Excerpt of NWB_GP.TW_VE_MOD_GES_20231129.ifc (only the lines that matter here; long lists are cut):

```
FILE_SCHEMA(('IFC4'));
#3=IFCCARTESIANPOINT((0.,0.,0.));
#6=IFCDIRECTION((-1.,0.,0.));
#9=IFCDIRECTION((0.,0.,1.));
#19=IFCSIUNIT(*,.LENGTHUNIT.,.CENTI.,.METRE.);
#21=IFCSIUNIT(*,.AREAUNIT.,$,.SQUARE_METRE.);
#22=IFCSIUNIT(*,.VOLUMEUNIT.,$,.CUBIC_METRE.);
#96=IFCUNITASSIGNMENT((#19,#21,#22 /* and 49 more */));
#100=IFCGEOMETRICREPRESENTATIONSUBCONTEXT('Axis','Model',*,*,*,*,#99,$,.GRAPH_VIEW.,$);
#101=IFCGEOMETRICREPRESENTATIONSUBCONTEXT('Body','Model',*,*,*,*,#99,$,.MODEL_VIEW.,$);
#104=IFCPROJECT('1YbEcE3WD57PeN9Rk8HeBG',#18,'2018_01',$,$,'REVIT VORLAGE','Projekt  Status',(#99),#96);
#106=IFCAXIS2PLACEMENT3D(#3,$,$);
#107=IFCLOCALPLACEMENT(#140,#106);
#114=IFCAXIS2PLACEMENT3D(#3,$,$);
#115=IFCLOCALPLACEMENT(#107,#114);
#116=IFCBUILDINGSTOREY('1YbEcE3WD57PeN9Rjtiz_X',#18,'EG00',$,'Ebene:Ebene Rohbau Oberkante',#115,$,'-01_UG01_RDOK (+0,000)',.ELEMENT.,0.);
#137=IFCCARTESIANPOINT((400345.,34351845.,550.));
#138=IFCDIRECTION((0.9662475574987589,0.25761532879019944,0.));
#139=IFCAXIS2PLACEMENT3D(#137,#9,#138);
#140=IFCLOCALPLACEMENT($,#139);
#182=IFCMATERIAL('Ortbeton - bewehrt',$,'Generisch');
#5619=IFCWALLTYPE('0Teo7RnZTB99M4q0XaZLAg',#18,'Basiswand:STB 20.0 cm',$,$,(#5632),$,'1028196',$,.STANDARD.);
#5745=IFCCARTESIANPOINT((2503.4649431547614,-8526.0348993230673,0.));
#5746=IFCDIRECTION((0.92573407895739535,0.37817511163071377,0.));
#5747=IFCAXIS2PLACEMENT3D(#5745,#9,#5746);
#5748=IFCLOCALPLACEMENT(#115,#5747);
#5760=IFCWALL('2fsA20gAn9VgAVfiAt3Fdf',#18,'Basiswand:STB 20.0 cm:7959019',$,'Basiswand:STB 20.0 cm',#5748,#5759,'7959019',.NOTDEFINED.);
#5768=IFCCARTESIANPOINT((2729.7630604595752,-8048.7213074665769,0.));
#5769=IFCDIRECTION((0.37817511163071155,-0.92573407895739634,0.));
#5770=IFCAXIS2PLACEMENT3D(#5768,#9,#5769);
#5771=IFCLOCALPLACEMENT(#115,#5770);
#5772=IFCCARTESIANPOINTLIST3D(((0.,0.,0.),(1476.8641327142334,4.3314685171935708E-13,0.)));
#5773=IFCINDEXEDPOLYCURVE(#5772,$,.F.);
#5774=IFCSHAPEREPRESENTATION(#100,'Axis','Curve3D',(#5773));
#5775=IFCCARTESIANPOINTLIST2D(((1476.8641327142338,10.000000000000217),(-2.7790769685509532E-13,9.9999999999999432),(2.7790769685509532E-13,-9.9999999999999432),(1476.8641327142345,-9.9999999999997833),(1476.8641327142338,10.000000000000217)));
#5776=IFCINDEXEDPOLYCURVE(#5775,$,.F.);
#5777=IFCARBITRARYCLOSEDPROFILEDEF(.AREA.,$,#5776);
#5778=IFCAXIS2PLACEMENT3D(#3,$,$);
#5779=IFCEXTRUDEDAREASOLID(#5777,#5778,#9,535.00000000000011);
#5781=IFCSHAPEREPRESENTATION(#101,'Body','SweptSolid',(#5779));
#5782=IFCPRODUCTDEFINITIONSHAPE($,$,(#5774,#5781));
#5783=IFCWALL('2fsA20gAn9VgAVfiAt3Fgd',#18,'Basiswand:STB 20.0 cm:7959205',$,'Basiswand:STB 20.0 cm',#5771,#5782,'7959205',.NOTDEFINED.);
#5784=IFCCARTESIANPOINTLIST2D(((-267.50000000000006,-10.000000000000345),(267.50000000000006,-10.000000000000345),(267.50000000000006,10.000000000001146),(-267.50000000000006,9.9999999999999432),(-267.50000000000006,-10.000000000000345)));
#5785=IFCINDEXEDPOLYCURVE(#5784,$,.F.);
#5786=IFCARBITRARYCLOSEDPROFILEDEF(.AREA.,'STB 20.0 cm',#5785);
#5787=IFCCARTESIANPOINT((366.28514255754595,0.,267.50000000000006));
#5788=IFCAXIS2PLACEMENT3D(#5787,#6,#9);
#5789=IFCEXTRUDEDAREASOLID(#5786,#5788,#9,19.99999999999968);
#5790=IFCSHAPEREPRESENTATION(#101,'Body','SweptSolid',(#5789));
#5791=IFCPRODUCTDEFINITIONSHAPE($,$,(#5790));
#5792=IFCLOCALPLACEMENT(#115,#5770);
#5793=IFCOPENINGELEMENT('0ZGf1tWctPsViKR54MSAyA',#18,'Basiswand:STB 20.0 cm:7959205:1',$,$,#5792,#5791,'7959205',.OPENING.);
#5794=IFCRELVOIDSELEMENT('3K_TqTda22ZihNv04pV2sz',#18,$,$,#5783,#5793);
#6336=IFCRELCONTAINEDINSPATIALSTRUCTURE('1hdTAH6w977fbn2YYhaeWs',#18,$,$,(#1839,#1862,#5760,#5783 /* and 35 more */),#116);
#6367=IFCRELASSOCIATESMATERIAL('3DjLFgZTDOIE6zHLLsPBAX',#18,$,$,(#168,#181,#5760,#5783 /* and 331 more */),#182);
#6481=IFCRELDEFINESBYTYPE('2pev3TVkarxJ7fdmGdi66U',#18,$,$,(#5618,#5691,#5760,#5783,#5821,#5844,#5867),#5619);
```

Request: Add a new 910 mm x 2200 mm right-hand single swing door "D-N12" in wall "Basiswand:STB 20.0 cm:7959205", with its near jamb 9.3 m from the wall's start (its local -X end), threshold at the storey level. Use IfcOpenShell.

```python
import numpy as np
import ifcopenshell
import ifcopenshell.api.feature
import ifcopenshell.api.geometry
import ifcopenshell.api.root
import ifcopenshell.api.spatial
import ifcopenshell.geom
import ifcopenshell.util.element
import ifcopenshell.util.placement
import ifcopenshell.util.representation
import ifcopenshell.util.shape
import ifcopenshell.util.unit

model = ifcopenshell.open("NWB_GP.TW_VE_MOD_GES_20231129.ifc")
unit_scale = ifcopenshell.util.unit.calculate_unit_scale(model)
settings = ifcopenshell.geom.settings()


def volume(element):
    """Net volume in cubic metres, openings subtracted."""
    shape = ifcopenshell.geom.create_shape(settings, element)
    return ifcopenshell.util.shape.get_volume(shape.geometry)


wall = model.by_guid("2fsA20gAn9VgAVfiAt3Fgd")
storey = ifcopenshell.util.element.get_container(wall, ifc_class="IfcBuildingStorey")
context = ifcopenshell.util.representation.get_context(model, "Model", "Body", "MODEL_VIEW")
before = volume(wall)

width, height, from_end, sill = 0.91, 2.2, 9.3, 0.0  # metres

# The wall runs along its own X axis, and the end named is its -X end.
wall_shape = ifcopenshell.geom.create_shape(settings, wall)
x, y, z = ifcopenshell.util.shape.get_vertices(wall_shape.geometry).T
start = x.min() + from_end
face, thickness = float(y.min()), float(y.max() - y.min())
wall_matrix = ifcopenshell.util.placement.get_local_placement(wall.ObjectPlacement)
level = ifcopenshell.util.placement.get_local_placement(storey.ObjectPlacement)[2, 3]


def in_wall(x, y):
    """Placement at x, y metres in the wall's axes, at sill height."""
    matrix = wall_matrix.copy()
    matrix[:, 3] = wall_matrix @ np.array([x / unit_scale, y / unit_scale, 0.0, 1.0])
    matrix[2, 3] = level + sill / unit_scale
    return matrix


# Opening: a box that overshoots both wall faces by 50 mm.
opening = ifcopenshell.api.root.create_entity(model, ifc_class="IfcOpeningElement", predefined_type="OPENING")
box = ifcopenshell.api.geometry.add_wall_representation(
    model, context=context, length=width, height=height, thickness=thickness + 0.1
)
ifcopenshell.api.geometry.assign_representation(model, product=opening, representation=box)
ifcopenshell.api.geometry.edit_object_placement(model, product=opening, matrix=in_wall(start, face - 0.05), is_si=False)
ifcopenshell.api.feature.add_feature(model, feature=opening, element=wall)

door = ifcopenshell.api.root.create_entity(model, ifc_class="IfcDoor", name="D-N12", predefined_type="DOOR")
door.OverallWidth, door.OverallHeight = width / unit_scale, height / unit_scale
door.OperationType = "SINGLE_SWING_RIGHT"
body = ifcopenshell.api.geometry.add_door_representation(
    model,
    context=context,
    overall_width=door.OverallWidth,
    overall_height=door.OverallHeight,
    operation_type="SINGLE_SWING_RIGHT",
    lining_properties={"LiningDepth": thickness / unit_scale, "ThresholdDepth": thickness / unit_scale},
)
ifcopenshell.api.geometry.assign_representation(model, product=door, representation=body)
ifcopenshell.api.spatial.assign_container(model, products=[door], relating_structure=storey)
ifcopenshell.api.feature.add_filling(model, opening=opening, element=door)

# The lining spans the wall, so the door starts at the wall face.
ifcopenshell.api.geometry.edit_object_placement(model, product=door, matrix=in_wall(start, face), is_si=False)

after = volume(wall)

print(f"wall volume {before:.3f} -> {after:.3f} m3")

model.write("NWB_GP.TW_VE_MOD_GES_20231129_edited.ifc")
```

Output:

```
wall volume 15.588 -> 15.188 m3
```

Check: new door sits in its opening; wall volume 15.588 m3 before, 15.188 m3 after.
